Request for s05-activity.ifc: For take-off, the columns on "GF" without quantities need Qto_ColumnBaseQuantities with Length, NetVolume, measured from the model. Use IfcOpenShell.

First a look at what the model holds.

```python
import ifcopenshell
import ifcopenshell.util.element
import ifcopenshell.util.unit

model = ifcopenshell.open("s05-activity.ifc")
print(model.schema)
for unit_type in ("LENGTHUNIT", "AREAUNIT", "VOLUMEUNIT"):
    print(unit_type, ifcopenshell.util.unit.calculate_unit_scale(model, unit_type))
storey = next(s for s in model.by_type("IfcBuildingStorey") if s.Name == "GF")
columns = [e for e in ifcopenshell.util.element.get_decomposition(storey) if e.is_a("IfcColumn")]
for e in sorted(columns, key=lambda e: e.id()):
    print(e.id(), e.is_a(), e.Name, list(ifcopenshell.util.element.get_psets(e, qtos_only=True)), sep=" | ")
```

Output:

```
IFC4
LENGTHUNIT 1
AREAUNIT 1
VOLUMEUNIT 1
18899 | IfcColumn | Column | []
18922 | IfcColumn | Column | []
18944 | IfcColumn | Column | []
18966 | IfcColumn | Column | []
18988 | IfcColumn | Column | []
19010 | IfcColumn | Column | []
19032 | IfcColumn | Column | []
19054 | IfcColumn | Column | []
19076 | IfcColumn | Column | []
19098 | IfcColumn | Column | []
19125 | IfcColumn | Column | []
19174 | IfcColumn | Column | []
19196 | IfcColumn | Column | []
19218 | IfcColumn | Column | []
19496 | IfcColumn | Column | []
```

```python
import ifcopenshell
import ifcopenshell.api.pset
import ifcopenshell.geom
import ifcopenshell.util.element
import ifcopenshell.util.shape
import ifcopenshell.util.unit

model = ifcopenshell.open("s05-activity.ifc")
unit_scale = ifcopenshell.util.unit.calculate_unit_scale(model)
volume_scale = ifcopenshell.util.unit.calculate_unit_scale(model, "VOLUMEUNIT")
settings = ifcopenshell.geom.settings()

storey = next(s for s in model.by_type("IfcBuildingStorey") if s.Name == "GF")
columns = [e for e in ifcopenshell.util.element.get_decomposition(storey) if e.is_a("IfcColumn")]

for e in sorted(columns, key=lambda e: e.id()):
    if ifcopenshell.util.element.get_psets(e, qtos_only=True, should_inherit=False):
        continue
    # Geometry comes back in metres, in the element's own axes.
    shape = ifcopenshell.geom.create_shape(settings, e)
    values = {
        "Length": ifcopenshell.util.shape.get_z(shape.geometry) / unit_scale,
        "NetVolume": ifcopenshell.util.shape.get_volume(shape.geometry) / volume_scale,
    }
    qto = ifcopenshell.api.pset.add_qto(model, product=e, name="Qto_ColumnBaseQuantities")
    ifcopenshell.api.pset.edit_qto(model, qto=qto, properties=values)
    print(e.id(), {k: round(v, 3) for k, v in values.items()})

model.write("s05-activity-out.ifc")
```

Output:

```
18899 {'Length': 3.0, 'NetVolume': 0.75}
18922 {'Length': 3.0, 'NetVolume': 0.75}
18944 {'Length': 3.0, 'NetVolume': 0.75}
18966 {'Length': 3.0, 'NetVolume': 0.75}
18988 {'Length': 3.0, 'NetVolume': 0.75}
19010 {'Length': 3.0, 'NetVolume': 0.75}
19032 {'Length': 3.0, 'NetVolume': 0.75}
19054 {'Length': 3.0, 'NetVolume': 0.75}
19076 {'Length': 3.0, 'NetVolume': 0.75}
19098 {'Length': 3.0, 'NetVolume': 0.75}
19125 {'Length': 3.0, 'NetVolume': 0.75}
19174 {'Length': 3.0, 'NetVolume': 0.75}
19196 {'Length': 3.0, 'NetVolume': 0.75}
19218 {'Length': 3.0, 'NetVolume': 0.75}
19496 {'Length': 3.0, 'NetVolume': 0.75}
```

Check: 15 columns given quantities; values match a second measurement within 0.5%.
